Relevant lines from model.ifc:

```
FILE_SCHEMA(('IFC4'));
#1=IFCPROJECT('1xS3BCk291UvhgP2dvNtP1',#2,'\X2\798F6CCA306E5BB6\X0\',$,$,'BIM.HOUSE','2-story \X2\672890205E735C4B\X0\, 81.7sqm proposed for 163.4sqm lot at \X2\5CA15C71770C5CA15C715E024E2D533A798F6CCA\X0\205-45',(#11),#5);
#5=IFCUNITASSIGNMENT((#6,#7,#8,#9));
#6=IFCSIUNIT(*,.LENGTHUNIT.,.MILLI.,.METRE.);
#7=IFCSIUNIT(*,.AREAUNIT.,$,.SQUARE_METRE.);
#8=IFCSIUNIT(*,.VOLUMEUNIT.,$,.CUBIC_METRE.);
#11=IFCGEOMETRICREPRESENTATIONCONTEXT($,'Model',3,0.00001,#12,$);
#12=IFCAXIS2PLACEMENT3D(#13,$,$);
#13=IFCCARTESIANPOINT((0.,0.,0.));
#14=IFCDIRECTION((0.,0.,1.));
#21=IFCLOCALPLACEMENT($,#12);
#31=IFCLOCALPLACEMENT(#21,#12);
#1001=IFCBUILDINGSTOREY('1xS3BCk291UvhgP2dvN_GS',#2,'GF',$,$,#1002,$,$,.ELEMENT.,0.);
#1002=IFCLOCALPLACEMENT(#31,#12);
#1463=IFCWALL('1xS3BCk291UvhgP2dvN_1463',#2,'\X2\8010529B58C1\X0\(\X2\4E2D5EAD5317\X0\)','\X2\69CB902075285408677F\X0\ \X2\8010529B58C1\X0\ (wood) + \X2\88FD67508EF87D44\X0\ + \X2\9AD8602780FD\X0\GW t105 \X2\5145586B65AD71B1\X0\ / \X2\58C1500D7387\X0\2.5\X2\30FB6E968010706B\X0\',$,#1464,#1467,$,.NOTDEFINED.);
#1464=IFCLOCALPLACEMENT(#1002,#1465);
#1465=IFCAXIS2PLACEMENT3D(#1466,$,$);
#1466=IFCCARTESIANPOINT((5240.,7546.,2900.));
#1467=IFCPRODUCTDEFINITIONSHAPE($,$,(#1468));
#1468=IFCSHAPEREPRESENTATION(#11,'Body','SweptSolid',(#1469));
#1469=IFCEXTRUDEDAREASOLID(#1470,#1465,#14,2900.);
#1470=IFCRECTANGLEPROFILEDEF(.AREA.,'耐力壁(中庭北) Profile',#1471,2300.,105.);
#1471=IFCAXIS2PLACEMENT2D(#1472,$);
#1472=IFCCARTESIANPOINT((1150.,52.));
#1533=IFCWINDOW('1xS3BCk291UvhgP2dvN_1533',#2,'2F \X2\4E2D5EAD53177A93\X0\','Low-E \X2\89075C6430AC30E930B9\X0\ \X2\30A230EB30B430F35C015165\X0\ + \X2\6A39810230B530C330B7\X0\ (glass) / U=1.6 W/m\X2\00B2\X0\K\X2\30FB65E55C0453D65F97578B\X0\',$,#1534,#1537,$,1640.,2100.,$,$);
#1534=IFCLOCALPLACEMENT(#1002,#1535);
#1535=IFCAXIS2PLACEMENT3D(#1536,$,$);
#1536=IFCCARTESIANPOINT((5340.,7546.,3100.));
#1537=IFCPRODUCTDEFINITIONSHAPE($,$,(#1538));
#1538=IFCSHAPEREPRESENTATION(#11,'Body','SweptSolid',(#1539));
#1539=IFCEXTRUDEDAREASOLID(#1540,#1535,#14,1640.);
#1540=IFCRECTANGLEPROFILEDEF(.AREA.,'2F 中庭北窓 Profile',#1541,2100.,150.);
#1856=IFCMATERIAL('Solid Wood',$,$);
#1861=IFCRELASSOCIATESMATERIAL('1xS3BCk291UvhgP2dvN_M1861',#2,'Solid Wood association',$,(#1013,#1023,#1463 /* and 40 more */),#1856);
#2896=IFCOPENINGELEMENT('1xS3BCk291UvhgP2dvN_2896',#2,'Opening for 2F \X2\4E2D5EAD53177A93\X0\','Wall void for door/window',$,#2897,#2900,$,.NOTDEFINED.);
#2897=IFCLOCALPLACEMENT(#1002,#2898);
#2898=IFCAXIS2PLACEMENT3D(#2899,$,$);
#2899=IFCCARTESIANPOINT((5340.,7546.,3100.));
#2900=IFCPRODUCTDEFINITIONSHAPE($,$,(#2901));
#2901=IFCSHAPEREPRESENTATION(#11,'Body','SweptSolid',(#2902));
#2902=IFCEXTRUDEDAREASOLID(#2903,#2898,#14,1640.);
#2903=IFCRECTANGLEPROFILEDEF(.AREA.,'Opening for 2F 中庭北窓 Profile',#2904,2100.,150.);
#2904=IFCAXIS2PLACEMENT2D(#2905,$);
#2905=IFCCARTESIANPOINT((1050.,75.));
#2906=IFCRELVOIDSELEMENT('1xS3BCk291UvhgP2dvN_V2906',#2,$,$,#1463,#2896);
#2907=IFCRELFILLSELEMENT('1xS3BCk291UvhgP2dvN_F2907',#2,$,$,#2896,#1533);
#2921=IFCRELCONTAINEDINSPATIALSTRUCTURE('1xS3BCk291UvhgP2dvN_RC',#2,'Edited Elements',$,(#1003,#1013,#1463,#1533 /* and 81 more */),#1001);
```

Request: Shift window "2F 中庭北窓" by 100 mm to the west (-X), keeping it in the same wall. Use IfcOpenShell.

```python
import ifcopenshell
import ifcopenshell.api.geometry
import ifcopenshell.util.placement
import ifcopenshell.util.unit

model = ifcopenshell.open("model.ifc")
unit_scale = ifcopenshell.util.unit.calculate_unit_scale(model)

window = model.by_id(1533)
opening = window.FillsVoids[0].RelatingOpeningElement
wall = opening.VoidsElements[0].RelatingBuildingElement

wall_matrix = ifcopenshell.util.placement.get_local_placement(wall.ObjectPlacement)
shift = wall_matrix[:3, 0] * -0.1 / unit_scale
before = ifcopenshell.util.placement.get_local_placement(window.ObjectPlacement)[:3, 3].copy()

# The window is not placed relative to its opening, so move both.
for product in (opening, window):
    matrix = ifcopenshell.util.placement.get_local_placement(product.ObjectPlacement)
    matrix[:3, 3] += shift
    ifcopenshell.api.geometry.edit_object_placement(model, product=product, matrix=matrix, is_si=False)

after = ifcopenshell.util.placement.get_local_placement(window.ObjectPlacement)[:3, 3]
print("window moved by", (after - before).round(3) + 0.0)

model.write("model-out.ifc")
```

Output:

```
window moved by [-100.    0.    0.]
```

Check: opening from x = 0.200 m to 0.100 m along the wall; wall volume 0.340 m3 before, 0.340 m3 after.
